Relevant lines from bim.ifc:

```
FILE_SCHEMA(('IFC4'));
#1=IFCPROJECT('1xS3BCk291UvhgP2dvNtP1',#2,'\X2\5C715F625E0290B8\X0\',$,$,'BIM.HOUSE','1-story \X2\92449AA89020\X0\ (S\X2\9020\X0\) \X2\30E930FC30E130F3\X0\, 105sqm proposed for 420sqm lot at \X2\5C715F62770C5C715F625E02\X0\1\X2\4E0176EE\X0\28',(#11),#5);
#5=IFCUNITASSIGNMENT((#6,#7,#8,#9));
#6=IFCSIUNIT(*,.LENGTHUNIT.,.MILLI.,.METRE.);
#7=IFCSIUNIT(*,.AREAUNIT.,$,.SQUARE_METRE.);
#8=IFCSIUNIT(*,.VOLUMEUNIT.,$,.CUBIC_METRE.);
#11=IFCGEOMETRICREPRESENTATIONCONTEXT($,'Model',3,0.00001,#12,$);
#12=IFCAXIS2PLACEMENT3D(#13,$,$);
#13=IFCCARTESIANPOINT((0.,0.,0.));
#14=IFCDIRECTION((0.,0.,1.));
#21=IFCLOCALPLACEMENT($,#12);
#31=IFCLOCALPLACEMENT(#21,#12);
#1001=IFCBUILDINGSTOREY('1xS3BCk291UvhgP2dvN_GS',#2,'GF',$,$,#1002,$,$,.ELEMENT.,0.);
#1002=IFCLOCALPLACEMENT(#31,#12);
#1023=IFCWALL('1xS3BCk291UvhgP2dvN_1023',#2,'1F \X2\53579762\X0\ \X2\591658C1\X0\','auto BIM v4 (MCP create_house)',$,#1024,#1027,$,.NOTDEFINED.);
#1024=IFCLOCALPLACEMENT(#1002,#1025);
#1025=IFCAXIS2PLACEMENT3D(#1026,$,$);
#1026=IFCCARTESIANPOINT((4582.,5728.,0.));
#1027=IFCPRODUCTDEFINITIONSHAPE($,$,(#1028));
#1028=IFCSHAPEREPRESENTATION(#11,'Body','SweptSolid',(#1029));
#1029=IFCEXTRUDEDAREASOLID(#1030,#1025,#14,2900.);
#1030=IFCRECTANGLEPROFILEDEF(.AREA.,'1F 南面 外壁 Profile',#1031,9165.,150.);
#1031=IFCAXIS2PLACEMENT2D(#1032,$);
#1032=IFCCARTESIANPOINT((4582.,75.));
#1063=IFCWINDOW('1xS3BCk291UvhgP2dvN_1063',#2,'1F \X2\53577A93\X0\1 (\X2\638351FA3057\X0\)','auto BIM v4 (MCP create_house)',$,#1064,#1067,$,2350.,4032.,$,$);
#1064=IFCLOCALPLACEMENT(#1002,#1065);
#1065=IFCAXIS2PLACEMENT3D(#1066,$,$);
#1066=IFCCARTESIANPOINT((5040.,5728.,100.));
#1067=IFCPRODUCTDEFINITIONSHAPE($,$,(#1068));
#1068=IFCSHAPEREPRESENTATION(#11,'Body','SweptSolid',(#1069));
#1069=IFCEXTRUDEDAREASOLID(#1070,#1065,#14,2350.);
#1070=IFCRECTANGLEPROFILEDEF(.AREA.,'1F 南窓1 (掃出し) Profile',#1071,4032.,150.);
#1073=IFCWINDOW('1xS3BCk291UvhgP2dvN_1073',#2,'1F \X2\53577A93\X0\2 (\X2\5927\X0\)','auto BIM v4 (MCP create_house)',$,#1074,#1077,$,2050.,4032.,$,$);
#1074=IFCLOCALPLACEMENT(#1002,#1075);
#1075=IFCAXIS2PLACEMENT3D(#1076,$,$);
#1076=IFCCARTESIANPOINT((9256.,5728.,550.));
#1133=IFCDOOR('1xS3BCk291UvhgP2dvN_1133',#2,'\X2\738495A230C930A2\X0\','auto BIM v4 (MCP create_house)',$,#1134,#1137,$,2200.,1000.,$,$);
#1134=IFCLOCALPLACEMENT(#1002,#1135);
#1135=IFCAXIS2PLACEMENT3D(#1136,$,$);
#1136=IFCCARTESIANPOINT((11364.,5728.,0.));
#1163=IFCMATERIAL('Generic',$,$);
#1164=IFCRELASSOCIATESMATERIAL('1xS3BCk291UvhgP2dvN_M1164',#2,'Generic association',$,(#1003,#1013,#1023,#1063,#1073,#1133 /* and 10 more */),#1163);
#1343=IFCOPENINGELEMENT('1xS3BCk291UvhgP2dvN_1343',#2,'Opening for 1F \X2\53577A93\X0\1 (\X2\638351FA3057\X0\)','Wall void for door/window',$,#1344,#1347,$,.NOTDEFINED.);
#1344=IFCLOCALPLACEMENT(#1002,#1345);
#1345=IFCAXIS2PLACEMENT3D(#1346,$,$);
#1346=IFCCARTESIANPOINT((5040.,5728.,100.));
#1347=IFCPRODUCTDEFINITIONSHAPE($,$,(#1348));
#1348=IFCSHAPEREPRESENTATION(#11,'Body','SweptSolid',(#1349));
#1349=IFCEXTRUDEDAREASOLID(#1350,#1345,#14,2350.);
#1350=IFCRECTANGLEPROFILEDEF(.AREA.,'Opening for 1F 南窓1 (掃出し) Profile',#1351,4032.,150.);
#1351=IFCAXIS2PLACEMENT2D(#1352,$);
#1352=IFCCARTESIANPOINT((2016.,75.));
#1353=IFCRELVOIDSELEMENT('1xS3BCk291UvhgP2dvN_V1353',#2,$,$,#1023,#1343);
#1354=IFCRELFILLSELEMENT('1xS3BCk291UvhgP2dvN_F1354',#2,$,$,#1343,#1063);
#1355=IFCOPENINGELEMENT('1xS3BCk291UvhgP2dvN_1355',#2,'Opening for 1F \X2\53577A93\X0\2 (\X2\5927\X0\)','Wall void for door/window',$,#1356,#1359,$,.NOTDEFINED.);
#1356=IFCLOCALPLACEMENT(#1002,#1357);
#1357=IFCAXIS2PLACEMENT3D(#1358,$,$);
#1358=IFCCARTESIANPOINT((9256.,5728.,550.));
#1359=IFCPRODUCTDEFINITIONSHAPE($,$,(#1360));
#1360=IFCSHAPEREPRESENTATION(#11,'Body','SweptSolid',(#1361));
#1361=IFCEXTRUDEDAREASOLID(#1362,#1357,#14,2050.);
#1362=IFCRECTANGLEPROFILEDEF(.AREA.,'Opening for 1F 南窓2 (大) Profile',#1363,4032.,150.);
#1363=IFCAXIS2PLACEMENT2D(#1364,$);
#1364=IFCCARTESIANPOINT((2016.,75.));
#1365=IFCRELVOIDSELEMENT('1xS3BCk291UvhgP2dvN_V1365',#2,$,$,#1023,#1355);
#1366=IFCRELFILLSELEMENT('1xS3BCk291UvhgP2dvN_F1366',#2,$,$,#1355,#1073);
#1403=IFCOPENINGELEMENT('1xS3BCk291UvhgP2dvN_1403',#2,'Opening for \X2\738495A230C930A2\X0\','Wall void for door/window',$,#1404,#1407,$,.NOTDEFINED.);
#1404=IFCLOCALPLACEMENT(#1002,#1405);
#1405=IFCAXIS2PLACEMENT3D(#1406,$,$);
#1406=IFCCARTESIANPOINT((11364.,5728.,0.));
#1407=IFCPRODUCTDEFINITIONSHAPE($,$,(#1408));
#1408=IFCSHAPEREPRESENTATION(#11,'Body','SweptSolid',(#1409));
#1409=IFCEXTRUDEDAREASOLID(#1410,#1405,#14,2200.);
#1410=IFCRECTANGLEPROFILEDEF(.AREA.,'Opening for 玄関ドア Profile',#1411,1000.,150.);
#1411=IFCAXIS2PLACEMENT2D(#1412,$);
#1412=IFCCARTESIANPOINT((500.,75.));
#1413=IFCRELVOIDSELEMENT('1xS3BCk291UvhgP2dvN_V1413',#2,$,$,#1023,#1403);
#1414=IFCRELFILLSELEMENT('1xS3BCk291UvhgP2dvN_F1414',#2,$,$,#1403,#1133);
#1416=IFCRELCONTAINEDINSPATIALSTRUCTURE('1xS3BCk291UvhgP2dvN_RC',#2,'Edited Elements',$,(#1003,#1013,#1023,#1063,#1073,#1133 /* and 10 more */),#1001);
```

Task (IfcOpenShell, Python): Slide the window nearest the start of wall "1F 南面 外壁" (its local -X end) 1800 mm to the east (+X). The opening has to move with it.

```python
import ifcopenshell
import ifcopenshell.api.geometry
import ifcopenshell.util.placement
import ifcopenshell.util.unit

model = ifcopenshell.open("bim.ifc")
unit_scale = ifcopenshell.util.unit.calculate_unit_scale(model)

window = model.by_guid("1xS3BCk291UvhgP2dvN_1063")
opening = window.FillsVoids[0].RelatingOpeningElement
wall = opening.VoidsElements[0].RelatingBuildingElement

wall_matrix = ifcopenshell.util.placement.get_local_placement(wall.ObjectPlacement)
shift = wall_matrix[:3, 0] * 1.8 / unit_scale
before = ifcopenshell.util.placement.get_local_placement(window.ObjectPlacement)[:3, 3].copy()

# The window is not placed relative to its opening, so move both.
for product in (opening, window):
    matrix = ifcopenshell.util.placement.get_local_placement(product.ObjectPlacement)
    matrix[:3, 3] += shift
    ifcopenshell.api.geometry.edit_object_placement(model, product=product, matrix=matrix, is_si=False)

after = ifcopenshell.util.placement.get_local_placement(window.ObjectPlacement)[:3, 3]
print("window moved by", (after - before).round(3) + 0.0)

model.write("bim_edited.ifc")
```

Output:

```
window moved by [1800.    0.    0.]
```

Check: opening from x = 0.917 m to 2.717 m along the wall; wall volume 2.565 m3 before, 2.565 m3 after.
